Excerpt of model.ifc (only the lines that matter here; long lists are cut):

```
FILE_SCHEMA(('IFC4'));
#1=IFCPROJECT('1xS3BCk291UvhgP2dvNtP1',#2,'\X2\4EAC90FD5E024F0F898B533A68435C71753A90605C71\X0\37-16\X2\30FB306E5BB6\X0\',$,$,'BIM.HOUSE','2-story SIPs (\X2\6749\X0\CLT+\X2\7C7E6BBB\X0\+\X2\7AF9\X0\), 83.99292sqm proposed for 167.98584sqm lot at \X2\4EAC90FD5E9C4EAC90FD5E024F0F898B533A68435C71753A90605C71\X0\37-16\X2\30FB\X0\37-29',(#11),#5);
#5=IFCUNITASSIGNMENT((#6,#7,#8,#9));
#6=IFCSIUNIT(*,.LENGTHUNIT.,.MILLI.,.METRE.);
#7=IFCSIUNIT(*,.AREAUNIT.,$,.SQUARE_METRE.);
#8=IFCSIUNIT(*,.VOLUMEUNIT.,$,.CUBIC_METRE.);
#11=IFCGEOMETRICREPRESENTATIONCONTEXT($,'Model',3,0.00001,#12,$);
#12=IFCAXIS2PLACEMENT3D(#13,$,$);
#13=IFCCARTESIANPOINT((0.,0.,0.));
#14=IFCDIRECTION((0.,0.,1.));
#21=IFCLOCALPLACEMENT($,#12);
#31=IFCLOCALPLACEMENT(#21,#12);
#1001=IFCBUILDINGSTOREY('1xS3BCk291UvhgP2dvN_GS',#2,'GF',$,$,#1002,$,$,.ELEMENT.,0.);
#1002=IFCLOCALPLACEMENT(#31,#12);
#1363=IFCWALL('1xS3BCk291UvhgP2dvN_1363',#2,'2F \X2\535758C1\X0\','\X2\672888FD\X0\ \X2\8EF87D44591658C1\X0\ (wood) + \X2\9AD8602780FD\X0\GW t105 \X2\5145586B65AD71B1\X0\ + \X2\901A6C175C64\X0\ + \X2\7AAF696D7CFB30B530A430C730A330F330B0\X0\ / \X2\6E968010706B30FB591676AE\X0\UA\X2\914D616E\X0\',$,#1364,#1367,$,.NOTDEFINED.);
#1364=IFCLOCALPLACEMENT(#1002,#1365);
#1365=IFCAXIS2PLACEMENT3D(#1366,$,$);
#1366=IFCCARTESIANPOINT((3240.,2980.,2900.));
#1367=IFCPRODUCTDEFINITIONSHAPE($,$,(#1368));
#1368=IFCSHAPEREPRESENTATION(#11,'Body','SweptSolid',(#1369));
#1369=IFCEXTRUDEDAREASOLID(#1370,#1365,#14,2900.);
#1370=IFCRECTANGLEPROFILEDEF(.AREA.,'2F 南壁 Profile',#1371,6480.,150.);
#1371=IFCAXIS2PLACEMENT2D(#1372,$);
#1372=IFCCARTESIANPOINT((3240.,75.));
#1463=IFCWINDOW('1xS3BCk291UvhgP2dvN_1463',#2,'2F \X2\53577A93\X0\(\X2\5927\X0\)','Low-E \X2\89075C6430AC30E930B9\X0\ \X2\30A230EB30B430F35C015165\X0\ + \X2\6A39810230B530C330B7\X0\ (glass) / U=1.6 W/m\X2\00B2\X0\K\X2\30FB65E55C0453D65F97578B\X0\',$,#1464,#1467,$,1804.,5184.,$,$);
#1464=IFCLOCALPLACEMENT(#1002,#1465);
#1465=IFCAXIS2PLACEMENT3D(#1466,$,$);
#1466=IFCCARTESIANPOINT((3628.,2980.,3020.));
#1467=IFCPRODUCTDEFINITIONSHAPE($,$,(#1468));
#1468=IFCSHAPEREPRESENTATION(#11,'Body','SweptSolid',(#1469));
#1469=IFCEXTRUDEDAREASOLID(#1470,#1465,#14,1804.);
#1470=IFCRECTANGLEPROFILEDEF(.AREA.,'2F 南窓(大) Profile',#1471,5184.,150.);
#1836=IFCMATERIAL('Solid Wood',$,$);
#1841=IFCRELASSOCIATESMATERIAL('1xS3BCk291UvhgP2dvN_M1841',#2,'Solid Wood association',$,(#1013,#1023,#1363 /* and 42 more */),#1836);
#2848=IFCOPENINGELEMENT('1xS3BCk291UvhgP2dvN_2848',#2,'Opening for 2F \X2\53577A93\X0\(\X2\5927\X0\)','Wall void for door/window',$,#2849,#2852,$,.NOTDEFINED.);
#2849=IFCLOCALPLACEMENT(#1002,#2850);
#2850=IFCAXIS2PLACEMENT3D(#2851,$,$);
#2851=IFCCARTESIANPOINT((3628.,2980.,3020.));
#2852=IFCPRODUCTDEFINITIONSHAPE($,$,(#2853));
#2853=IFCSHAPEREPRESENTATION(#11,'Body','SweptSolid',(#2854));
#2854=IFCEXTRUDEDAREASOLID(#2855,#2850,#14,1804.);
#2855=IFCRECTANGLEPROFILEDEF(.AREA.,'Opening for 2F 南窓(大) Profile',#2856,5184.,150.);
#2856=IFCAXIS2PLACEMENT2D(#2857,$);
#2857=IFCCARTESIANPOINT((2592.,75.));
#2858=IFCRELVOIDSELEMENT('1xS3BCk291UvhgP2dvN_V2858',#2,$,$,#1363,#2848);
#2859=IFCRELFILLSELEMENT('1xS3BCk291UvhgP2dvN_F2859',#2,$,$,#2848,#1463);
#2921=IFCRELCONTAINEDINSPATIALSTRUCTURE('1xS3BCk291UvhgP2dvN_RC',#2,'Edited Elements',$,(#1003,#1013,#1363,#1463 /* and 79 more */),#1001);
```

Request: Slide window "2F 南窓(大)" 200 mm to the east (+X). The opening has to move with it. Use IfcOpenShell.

```python
import ifcopenshell
import ifcopenshell.api.geometry
import ifcopenshell.util.placement
import ifcopenshell.util.unit

model = ifcopenshell.open("model.ifc")
unit_scale = ifcopenshell.util.unit.calculate_unit_scale(model)

window = model.by_id(1463)
opening = window.FillsVoids[0].RelatingOpeningElement
wall = opening.VoidsElements[0].RelatingBuildingElement

wall_matrix = ifcopenshell.util.placement.get_local_placement(wall.ObjectPlacement)
shift = wall_matrix[:3, 0] * 0.2 / unit_scale
before = ifcopenshell.util.placement.get_local_placement(window.ObjectPlacement)[:3, 3].copy()

# The window is not placed relative to its opening, so move both.
for product in (opening, window):
    matrix = ifcopenshell.util.placement.get_local_placement(product.ObjectPlacement)
    matrix[:3, 3] += shift
    ifcopenshell.api.geometry.edit_object_placement(model, product=product, matrix=matrix, is_si=False)

after = ifcopenshell.util.placement.get_local_placement(window.ObjectPlacement)[:3, 3]
print("window moved by", (after - before).round(3) + 0.0)

model.write("model_updated.ifc")
```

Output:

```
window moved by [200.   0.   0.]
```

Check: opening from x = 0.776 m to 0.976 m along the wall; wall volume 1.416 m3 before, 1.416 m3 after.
